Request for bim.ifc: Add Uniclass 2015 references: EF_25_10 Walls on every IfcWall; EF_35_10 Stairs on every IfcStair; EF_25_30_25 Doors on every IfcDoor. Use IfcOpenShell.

First a look at what the model holds.

```python
import ifcopenshell

model = ifcopenshell.open("bim.ifc")
print(model.schema)
print("classifications:", [c.Name for c in model.by_type("IfcClassification")])
for ifc_class in ("IfcDoor", "IfcRoof", "IfcStair", "IfcWall", "IfcWindow"):
    print(ifc_class, len(model.by_type(ifc_class)))
```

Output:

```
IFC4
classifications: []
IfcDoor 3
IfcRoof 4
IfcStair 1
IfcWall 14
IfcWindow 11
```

```python
import ifcopenshell
import ifcopenshell.api.classification

model = ifcopenshell.open("bim.ifc")

system = ifcopenshell.api.classification.add_classification(model, classification="Uniclass 2015")

codes = {
    "IfcWall": ("EF_25_10", "Walls"),
    "IfcStair": ("EF_35_10", "Stairs"),
    "IfcDoor": ("EF_25_30_25", "Doors"),
}
for ifc_class, (code, name) in codes.items():
    products = model.by_type(ifc_class)
    ifcopenshell.api.classification.add_reference(
        model, products=products, classification=system, identification=code, name=name
    )
    print(code, len(products))

model.write("bim-out.ifc")
```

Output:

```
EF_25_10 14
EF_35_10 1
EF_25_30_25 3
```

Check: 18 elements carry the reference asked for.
